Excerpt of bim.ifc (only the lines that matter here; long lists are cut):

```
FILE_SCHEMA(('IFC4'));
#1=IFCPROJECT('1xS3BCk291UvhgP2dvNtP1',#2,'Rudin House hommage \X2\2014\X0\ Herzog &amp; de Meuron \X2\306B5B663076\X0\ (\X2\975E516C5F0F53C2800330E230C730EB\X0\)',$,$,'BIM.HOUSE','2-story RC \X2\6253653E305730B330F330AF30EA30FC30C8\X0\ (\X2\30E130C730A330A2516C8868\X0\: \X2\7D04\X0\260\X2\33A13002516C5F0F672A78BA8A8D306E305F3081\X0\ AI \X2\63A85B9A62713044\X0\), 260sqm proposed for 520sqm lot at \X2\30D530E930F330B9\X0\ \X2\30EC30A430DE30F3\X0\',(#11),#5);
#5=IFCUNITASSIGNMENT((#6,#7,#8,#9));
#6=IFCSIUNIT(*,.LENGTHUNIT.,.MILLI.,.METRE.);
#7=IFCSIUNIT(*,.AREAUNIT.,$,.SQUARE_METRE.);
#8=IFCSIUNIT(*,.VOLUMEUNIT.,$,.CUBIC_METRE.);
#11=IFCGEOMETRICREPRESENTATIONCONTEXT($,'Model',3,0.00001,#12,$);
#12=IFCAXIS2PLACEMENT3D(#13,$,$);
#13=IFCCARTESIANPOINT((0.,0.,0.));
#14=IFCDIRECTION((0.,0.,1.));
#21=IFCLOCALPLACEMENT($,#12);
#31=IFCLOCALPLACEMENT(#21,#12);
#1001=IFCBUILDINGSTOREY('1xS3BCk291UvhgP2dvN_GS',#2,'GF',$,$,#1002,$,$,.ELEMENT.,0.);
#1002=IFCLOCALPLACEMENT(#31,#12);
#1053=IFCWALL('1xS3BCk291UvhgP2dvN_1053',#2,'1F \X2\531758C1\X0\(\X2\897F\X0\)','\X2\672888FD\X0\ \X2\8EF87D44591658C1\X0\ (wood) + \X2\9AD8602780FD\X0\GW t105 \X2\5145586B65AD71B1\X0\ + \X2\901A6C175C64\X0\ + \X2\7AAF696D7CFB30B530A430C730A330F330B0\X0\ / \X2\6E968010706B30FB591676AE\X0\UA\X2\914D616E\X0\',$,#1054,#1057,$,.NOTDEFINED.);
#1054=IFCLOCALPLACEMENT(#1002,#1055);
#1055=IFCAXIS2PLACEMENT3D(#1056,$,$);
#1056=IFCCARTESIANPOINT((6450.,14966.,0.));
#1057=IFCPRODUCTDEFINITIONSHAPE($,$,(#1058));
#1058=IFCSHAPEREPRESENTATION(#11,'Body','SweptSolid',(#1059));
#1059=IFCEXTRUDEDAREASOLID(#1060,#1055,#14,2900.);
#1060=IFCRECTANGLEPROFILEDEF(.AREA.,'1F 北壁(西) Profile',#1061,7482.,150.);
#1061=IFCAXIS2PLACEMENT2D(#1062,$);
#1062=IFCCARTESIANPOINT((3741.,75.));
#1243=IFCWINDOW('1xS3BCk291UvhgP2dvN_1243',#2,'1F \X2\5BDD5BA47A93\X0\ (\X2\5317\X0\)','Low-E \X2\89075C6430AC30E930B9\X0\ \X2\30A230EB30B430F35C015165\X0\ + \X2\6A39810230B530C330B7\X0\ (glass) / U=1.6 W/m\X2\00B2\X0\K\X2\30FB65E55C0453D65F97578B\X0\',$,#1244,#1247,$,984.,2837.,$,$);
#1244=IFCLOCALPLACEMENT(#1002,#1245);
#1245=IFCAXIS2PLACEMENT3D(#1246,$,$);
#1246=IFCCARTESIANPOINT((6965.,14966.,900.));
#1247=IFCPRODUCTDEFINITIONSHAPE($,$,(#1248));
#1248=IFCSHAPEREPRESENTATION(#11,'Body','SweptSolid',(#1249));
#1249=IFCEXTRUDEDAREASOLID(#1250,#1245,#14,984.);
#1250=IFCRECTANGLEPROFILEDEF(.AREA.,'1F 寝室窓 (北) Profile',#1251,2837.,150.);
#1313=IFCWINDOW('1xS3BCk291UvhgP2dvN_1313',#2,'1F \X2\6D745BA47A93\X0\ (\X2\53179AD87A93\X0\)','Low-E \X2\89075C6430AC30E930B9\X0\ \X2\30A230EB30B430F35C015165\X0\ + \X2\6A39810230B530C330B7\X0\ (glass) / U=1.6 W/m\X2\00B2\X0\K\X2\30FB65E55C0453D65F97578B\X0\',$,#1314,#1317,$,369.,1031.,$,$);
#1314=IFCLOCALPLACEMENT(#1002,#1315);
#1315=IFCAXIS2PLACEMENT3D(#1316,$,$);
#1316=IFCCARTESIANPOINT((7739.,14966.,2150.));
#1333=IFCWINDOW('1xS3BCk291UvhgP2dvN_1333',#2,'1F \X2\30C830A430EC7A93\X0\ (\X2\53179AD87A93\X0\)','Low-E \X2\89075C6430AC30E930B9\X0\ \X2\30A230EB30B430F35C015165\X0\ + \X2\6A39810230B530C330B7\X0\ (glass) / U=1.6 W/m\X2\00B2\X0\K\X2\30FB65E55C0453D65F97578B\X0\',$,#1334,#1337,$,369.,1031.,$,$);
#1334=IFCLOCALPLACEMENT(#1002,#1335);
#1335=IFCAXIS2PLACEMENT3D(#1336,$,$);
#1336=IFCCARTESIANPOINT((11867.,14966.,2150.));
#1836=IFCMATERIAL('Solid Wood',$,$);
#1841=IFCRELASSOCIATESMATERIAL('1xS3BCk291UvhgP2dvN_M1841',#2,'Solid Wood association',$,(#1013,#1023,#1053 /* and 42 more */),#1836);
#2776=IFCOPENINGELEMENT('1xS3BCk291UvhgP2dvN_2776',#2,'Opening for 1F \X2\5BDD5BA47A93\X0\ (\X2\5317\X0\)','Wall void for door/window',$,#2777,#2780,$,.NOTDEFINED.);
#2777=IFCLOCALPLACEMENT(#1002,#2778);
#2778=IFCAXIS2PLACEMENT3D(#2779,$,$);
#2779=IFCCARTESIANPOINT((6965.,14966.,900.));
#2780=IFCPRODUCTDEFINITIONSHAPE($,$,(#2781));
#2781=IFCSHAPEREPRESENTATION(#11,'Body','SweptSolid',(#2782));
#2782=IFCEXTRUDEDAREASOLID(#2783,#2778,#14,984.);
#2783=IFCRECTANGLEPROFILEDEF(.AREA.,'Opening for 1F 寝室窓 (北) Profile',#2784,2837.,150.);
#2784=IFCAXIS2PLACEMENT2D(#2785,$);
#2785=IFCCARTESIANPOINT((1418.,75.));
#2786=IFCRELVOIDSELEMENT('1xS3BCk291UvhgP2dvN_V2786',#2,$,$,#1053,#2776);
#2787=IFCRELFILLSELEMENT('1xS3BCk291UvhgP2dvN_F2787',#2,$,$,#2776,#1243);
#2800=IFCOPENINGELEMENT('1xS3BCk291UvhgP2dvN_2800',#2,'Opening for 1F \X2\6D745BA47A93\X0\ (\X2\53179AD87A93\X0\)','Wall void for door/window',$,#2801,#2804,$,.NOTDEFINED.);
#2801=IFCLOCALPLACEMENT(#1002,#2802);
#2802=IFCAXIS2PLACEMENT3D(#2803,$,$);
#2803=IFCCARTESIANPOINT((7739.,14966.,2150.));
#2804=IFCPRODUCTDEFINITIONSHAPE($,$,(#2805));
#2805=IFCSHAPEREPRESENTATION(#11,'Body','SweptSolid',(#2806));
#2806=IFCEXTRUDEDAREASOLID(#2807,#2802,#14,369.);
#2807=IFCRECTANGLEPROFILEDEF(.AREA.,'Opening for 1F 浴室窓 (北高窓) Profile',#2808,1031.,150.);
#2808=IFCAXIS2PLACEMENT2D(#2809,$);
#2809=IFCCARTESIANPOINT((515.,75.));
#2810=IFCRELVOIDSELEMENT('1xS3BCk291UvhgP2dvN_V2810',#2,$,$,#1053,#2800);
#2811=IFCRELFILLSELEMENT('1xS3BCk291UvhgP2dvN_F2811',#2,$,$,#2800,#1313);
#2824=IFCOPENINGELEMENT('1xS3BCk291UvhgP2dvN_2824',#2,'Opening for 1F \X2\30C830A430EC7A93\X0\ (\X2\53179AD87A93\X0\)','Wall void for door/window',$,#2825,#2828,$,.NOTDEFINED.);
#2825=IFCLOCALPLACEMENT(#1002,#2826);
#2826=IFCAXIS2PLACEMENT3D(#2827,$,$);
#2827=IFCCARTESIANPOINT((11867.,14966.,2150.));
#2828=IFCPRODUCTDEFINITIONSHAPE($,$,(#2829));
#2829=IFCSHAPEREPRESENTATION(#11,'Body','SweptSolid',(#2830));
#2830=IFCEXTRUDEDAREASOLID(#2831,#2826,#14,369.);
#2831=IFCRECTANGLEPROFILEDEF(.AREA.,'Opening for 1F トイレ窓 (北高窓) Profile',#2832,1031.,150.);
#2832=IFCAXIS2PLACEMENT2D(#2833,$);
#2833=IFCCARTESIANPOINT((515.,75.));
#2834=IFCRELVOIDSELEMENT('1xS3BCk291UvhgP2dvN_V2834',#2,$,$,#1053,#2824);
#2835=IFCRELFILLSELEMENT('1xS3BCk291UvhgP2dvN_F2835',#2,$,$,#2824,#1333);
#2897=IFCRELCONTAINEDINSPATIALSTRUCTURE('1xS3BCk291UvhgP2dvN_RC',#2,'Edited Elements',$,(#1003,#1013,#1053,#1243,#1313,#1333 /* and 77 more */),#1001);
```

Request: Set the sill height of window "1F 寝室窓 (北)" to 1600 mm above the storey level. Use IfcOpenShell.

```python
import numpy as np
import ifcopenshell
import ifcopenshell.api.geometry
import ifcopenshell.geom
import ifcopenshell.util.element
import ifcopenshell.util.placement
import ifcopenshell.util.shape
import ifcopenshell.util.unit

model = ifcopenshell.open("bim.ifc")
unit_scale = ifcopenshell.util.unit.calculate_unit_scale(model)

window = model.by_id(1243)
opening = window.FillsVoids[0].RelatingOpeningElement
storey = ifcopenshell.util.element.get_container(window, ifc_class="IfcBuildingStorey")
level = ifcopenshell.util.placement.get_local_placement(storey.ObjectPlacement)[2, 3]

# The opening's origin need not be at the sill, so measure its lowest point.
shape = ifcopenshell.geom.create_shape(ifcopenshell.geom.settings(), opening)
bottom = ifcopenshell.util.shape.get_shape_bottom_elevation(shape, shape.geometry) / unit_scale
dz = level + 1.6 / unit_scale - bottom

shift = np.array([0.0, 0.0, dz])
# The window is not placed relative to its opening, so move both.
for product in (opening, window):
    matrix = ifcopenshell.util.placement.get_local_placement(product.ObjectPlacement)
    matrix[:3, 3] += shift
    ifcopenshell.api.geometry.edit_object_placement(model, product=product, matrix=matrix, is_si=False)

print(f"moved by {dz * unit_scale:+.3f} m")

model.write("bim_edited.ifc")
```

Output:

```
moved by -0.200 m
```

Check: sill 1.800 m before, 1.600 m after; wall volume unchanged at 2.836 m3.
